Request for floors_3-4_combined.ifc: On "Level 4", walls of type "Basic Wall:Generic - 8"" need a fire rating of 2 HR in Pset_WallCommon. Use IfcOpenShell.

First a look at what the model holds.

```python
import ifcopenshell
import ifcopenshell.util.element

model = ifcopenshell.open("floors_3-4_combined.ifc")
print(model.schema)
storey = next(s for s in model.by_type("IfcBuildingStorey") if s.Name == "Level 4")
walls = [e for e in ifcopenshell.util.element.get_decomposition(storey) if e.is_a("IfcWall")]
seen = {}
for e in walls:
    element_type = ifcopenshell.util.element.get_type(e)
    key = (element_type.Name if element_type != e and element_type else None, ifcopenshell.util.element.get_pset(e, "Pset_WallCommon", "FireRating"))
    seen[key] = seen.get(key, 0) + 1
for (name, value), count in sorted(seen.items(), key=str):
    print(count, "x", name, "|", value)
```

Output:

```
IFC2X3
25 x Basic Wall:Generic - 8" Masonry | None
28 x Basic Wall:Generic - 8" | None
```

```python
import ifcopenshell
import ifcopenshell.api.pset
import ifcopenshell.util.element

model = ifcopenshell.open("floors_3-4_combined.ifc")

storey = next(s for s in model.by_type("IfcBuildingStorey") if s.Name == "Level 4")
walls = [e for e in ifcopenshell.util.element.get_decomposition(storey) if e.is_a("IfcWall")]

count = 0
for e in walls:
    element_type = ifcopenshell.util.element.get_type(e)
    if element_type in (None, e) or element_type.Name != 'Basic Wall:Generic - 8"':
        continue
    # add_pset returns the element's existing set when there is one.
    pset = ifcopenshell.api.pset.add_pset(model, product=e, name="Pset_WallCommon")
    ifcopenshell.api.pset.edit_pset(model, pset=pset, properties={"FireRating": "2 HR"})
    count += 1

print(count, "walls updated")

model.write("floors_3-4_combined_updated.ifc")
```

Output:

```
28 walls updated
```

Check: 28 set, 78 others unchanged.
